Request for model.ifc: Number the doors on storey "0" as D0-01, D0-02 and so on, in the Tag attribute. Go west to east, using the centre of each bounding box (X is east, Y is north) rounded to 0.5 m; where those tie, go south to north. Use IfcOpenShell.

First a look at what the model holds.

```python
import ifcopenshell
import ifcopenshell.util.element
import ifcopenshell.util.placement

model = ifcopenshell.open("model.ifc")
print(model.schema)
storey = next(s for s in model.by_type("IfcBuildingStorey") if s.Name == "0")
doors = [e for e in ifcopenshell.util.element.get_decomposition(storey) if e.is_a("IfcDoor")]
for e in sorted(doors, key=lambda e: e.id()):
    origin = ifcopenshell.util.placement.get_local_placement(e.ObjectPlacement)[:3, 3]
    print(e.id(), e.Tag, e.Name, origin.round(2) + 0.0, sep=" | ")
```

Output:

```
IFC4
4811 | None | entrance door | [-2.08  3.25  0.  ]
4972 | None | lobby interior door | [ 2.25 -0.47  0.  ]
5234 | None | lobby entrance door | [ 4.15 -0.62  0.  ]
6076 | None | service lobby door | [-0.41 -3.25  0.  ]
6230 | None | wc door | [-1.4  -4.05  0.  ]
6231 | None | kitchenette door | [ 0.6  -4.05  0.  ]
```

```python
import ifcopenshell
import ifcopenshell.geom
import ifcopenshell.util.element
import ifcopenshell.util.shape

model = ifcopenshell.open("model.ifc")
settings = ifcopenshell.geom.settings()
settings.set("use-world-coords", True)


def centre(element):
    shape = ifcopenshell.geom.create_shape(settings, element)
    return ifcopenshell.util.shape.get_bbox_centroid(shape.geometry)


storey = next(s for s in model.by_type("IfcBuildingStorey") if s.Name == "0")
doors = [e for e in ifcopenshell.util.element.get_decomposition(storey) if e.is_a("IfcDoor")]

# Insertion points can sit at a corner or the storey origin, so sort by the geometry (in metres).
centres = {e: centre(e) for e in doors}
doors.sort(key=lambda e: (round(centres[e][0] / 0.5), centres[e][1]))

for i, e in enumerate(doors, start=1):
    number = f"D0-{i:02d}"
    e.Tag = number
    print(e.id(), number)

model.write("model_v2.ifc")
```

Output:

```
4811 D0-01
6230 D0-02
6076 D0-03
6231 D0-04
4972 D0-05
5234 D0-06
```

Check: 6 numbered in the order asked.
